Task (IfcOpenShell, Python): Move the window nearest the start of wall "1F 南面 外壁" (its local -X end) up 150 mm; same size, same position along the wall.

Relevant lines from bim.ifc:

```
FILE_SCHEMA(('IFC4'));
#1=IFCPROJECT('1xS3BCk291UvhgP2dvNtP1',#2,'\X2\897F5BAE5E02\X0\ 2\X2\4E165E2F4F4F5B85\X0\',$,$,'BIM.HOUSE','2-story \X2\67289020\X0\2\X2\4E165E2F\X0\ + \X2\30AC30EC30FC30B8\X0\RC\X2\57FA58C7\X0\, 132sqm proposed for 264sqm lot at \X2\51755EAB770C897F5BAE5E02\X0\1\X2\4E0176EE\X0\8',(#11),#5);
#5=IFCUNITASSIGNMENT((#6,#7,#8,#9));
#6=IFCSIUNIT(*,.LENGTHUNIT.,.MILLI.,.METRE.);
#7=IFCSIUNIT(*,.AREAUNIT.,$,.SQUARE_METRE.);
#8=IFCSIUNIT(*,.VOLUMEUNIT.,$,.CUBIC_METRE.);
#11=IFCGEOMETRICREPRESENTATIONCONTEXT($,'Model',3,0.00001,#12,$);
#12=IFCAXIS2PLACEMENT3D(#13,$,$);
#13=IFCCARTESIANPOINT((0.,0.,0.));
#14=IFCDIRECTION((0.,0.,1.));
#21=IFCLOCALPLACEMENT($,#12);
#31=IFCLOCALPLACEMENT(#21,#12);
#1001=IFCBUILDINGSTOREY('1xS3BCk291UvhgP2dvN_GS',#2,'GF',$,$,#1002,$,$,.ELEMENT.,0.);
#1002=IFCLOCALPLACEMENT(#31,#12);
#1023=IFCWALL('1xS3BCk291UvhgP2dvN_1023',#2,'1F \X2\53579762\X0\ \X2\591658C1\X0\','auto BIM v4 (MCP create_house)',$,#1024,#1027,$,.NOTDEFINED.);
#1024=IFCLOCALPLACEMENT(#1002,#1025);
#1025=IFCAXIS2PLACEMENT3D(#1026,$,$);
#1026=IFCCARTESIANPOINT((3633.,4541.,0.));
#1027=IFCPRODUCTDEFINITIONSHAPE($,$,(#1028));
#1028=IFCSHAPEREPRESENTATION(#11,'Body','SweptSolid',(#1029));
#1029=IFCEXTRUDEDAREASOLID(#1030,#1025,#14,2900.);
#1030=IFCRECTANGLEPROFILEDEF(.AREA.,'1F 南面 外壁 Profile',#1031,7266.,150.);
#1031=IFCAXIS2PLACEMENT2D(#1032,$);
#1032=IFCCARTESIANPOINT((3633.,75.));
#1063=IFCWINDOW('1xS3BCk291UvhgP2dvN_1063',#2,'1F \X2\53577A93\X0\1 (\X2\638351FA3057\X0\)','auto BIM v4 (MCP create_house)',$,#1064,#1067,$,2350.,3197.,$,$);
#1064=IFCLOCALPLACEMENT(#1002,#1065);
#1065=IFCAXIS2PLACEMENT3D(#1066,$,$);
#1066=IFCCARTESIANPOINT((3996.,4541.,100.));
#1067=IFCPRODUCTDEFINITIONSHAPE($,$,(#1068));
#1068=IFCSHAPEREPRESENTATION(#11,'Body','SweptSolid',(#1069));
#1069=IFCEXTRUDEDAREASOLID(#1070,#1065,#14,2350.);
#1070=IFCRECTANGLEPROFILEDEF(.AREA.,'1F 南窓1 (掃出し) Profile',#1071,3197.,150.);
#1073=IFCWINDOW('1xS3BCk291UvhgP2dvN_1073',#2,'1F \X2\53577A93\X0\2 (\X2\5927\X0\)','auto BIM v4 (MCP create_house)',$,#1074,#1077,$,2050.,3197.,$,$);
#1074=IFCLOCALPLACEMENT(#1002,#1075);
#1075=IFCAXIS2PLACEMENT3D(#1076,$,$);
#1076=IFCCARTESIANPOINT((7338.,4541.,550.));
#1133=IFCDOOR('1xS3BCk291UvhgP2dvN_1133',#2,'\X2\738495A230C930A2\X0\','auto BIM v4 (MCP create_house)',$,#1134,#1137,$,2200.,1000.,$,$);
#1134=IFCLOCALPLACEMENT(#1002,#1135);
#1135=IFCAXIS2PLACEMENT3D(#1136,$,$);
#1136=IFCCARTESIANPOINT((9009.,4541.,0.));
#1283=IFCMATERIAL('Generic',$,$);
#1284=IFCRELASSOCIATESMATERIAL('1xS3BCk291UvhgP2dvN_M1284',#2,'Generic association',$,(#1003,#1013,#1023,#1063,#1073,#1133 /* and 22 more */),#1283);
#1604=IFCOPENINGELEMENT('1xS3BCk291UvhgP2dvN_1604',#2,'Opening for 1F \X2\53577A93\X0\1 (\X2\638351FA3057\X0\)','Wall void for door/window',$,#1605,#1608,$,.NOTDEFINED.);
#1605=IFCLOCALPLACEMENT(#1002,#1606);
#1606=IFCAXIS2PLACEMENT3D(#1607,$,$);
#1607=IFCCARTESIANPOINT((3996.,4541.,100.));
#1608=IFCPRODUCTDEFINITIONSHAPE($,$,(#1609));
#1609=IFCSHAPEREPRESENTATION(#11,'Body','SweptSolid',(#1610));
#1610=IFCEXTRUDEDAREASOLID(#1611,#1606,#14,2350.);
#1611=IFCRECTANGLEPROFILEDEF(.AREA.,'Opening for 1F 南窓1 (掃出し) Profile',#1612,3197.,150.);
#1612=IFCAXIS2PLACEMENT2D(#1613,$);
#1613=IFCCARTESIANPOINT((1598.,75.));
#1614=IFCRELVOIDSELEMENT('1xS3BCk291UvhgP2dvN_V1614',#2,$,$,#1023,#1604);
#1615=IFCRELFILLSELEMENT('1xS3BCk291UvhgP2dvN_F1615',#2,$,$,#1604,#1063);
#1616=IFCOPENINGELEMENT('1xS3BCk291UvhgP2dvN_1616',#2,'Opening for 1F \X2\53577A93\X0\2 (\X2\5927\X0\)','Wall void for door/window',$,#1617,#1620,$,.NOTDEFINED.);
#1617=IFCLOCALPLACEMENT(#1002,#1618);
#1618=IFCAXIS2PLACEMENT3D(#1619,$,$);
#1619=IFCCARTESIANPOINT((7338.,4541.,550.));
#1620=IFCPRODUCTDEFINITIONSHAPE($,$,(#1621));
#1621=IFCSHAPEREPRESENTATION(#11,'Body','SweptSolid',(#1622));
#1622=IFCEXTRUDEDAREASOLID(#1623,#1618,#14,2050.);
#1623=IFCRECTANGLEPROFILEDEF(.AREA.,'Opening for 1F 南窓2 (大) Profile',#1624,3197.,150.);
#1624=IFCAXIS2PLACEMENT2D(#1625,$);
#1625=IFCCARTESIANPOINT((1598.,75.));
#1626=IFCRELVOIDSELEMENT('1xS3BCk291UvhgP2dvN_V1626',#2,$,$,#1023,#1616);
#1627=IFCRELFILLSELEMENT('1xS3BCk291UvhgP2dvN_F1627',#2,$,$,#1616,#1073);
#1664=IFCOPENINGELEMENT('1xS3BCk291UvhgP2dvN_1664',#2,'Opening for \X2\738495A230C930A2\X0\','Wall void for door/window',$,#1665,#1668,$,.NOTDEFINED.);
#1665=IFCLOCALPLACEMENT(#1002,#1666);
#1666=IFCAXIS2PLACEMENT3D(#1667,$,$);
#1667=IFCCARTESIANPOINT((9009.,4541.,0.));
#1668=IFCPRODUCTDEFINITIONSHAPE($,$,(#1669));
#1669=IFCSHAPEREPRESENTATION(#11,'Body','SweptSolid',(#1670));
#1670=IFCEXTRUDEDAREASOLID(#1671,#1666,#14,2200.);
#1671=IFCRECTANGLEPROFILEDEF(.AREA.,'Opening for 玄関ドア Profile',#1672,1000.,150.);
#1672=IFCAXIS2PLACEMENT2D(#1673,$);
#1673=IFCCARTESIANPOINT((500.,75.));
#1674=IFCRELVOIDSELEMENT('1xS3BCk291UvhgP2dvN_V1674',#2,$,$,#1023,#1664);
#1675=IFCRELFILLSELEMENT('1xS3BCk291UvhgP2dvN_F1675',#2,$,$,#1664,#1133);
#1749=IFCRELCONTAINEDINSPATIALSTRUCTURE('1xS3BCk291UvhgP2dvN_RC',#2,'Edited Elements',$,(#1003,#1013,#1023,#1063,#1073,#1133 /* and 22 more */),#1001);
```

```python
import numpy as np
import ifcopenshell
import ifcopenshell.api.geometry
import ifcopenshell.util.placement
import ifcopenshell.util.unit

model = ifcopenshell.open("bim.ifc")
unit_scale = ifcopenshell.util.unit.calculate_unit_scale(model)

window = model.by_guid("1xS3BCk291UvhgP2dvN_1063")
opening = window.FillsVoids[0].RelatingOpeningElement
dz = 150.0

shift = np.array([0.0, 0.0, dz])
# The window is not placed relative to its opening, so move both.
for product in (opening, window):
    matrix = ifcopenshell.util.placement.get_local_placement(product.ObjectPlacement)
    matrix[:3, 3] += shift
    ifcopenshell.api.geometry.edit_object_placement(model, product=product, matrix=matrix, is_si=False)

print(f"moved by {dz * unit_scale:+.3f} m")

model.write("bim-out.ifc")
```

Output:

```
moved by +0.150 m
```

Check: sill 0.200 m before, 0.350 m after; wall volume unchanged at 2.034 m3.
